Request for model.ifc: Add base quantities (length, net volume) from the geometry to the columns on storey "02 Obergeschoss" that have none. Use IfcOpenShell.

First a look at what the model holds.

```python
import ifcopenshell
import ifcopenshell.util.element
import ifcopenshell.util.unit

model = ifcopenshell.open("model.ifc")
print(model.schema)
for unit_type in ("LENGTHUNIT", "AREAUNIT", "VOLUMEUNIT"):
    print(unit_type, ifcopenshell.util.unit.calculate_unit_scale(model, unit_type))
storey = next(s for s in model.by_type("IfcBuildingStorey") if s.Name == "02 Obergeschoss")
columns = [e for e in ifcopenshell.util.element.get_decomposition(storey) if e.is_a("IfcColumn")]
for e in sorted(columns, key=lambda e: e.id()):
    print(e.id(), e.is_a(), e.Name, list(ifcopenshell.util.element.get_psets(e, qtos_only=True)), sep=" | ")
```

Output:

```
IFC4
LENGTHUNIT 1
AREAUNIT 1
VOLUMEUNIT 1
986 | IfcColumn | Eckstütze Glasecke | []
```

```python
import ifcopenshell
import ifcopenshell.api.pset
import ifcopenshell.geom
import ifcopenshell.util.element
import ifcopenshell.util.shape
import ifcopenshell.util.unit

model = ifcopenshell.open("model.ifc")
unit_scale = ifcopenshell.util.unit.calculate_unit_scale(model)
volume_scale = ifcopenshell.util.unit.calculate_unit_scale(model, "VOLUMEUNIT")
settings = ifcopenshell.geom.settings()

storey = next(s for s in model.by_type("IfcBuildingStorey") if s.Name == "02 Obergeschoss")
columns = [e for e in ifcopenshell.util.element.get_decomposition(storey) if e.is_a("IfcColumn")]

for e in sorted(columns, key=lambda e: e.id()):
    if ifcopenshell.util.element.get_psets(e, qtos_only=True, should_inherit=False):
        continue
    # Geometry comes back in metres, in the element's own axes.
    shape = ifcopenshell.geom.create_shape(settings, e)
    values = {
        "Length": ifcopenshell.util.shape.get_z(shape.geometry) / unit_scale,
        "NetVolume": ifcopenshell.util.shape.get_volume(shape.geometry) / volume_scale,
    }
    qto = ifcopenshell.api.pset.add_qto(model, product=e, name="Qto_ColumnBaseQuantities")
    ifcopenshell.api.pset.edit_qto(model, qto=qto, properties=values)
    print(e.id(), {k: round(v, 3) for k, v in values.items()})

model.write("model_v2.ifc")
```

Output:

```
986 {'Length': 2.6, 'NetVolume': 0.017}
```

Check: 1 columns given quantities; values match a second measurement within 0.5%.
